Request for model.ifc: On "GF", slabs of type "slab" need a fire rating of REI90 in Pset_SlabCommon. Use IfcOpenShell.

First a look at what the model holds.

```python
import ifcopenshell
import ifcopenshell.util.element

model = ifcopenshell.open("model.ifc")
print(model.schema)
storey = next(s for s in model.by_type("IfcBuildingStorey") if s.Name == "GF")
slabs = [e for e in ifcopenshell.util.element.get_decomposition(storey) if e.is_a("IfcSlab")]
seen = {}
for e in slabs:
    element_type = ifcopenshell.util.element.get_type(e)
    key = (element_type.Name if element_type != e and element_type else None, ifcopenshell.util.element.get_pset(e, "Pset_SlabCommon", "FireRating"))
    seen[key] = seen.get(key, 0) + 1
for (name, value), count in sorted(seen.items(), key=str):
    print(count, "x", name, "|", value)
```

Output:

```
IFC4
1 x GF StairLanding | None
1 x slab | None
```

```python
import ifcopenshell
import ifcopenshell.api.pset
import ifcopenshell.util.element

model = ifcopenshell.open("model.ifc")

storey = next(s for s in model.by_type("IfcBuildingStorey") if s.Name == "GF")
slabs = [e for e in ifcopenshell.util.element.get_decomposition(storey) if e.is_a("IfcSlab")]

count = 0
for e in slabs:
    element_type = ifcopenshell.util.element.get_type(e)
    if element_type in (None, e) or element_type.Name != "slab":
        continue
    # add_pset returns the element's existing set when there is one.
    pset = ifcopenshell.api.pset.add_pset(model, product=e, name="Pset_SlabCommon")
    ifcopenshell.api.pset.edit_pset(model, pset=pset, properties={"FireRating": "REI90"})
    count += 1

print(count, "slabs updated")

model.write("model_edited.ifc")
```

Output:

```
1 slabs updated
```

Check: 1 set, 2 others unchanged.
